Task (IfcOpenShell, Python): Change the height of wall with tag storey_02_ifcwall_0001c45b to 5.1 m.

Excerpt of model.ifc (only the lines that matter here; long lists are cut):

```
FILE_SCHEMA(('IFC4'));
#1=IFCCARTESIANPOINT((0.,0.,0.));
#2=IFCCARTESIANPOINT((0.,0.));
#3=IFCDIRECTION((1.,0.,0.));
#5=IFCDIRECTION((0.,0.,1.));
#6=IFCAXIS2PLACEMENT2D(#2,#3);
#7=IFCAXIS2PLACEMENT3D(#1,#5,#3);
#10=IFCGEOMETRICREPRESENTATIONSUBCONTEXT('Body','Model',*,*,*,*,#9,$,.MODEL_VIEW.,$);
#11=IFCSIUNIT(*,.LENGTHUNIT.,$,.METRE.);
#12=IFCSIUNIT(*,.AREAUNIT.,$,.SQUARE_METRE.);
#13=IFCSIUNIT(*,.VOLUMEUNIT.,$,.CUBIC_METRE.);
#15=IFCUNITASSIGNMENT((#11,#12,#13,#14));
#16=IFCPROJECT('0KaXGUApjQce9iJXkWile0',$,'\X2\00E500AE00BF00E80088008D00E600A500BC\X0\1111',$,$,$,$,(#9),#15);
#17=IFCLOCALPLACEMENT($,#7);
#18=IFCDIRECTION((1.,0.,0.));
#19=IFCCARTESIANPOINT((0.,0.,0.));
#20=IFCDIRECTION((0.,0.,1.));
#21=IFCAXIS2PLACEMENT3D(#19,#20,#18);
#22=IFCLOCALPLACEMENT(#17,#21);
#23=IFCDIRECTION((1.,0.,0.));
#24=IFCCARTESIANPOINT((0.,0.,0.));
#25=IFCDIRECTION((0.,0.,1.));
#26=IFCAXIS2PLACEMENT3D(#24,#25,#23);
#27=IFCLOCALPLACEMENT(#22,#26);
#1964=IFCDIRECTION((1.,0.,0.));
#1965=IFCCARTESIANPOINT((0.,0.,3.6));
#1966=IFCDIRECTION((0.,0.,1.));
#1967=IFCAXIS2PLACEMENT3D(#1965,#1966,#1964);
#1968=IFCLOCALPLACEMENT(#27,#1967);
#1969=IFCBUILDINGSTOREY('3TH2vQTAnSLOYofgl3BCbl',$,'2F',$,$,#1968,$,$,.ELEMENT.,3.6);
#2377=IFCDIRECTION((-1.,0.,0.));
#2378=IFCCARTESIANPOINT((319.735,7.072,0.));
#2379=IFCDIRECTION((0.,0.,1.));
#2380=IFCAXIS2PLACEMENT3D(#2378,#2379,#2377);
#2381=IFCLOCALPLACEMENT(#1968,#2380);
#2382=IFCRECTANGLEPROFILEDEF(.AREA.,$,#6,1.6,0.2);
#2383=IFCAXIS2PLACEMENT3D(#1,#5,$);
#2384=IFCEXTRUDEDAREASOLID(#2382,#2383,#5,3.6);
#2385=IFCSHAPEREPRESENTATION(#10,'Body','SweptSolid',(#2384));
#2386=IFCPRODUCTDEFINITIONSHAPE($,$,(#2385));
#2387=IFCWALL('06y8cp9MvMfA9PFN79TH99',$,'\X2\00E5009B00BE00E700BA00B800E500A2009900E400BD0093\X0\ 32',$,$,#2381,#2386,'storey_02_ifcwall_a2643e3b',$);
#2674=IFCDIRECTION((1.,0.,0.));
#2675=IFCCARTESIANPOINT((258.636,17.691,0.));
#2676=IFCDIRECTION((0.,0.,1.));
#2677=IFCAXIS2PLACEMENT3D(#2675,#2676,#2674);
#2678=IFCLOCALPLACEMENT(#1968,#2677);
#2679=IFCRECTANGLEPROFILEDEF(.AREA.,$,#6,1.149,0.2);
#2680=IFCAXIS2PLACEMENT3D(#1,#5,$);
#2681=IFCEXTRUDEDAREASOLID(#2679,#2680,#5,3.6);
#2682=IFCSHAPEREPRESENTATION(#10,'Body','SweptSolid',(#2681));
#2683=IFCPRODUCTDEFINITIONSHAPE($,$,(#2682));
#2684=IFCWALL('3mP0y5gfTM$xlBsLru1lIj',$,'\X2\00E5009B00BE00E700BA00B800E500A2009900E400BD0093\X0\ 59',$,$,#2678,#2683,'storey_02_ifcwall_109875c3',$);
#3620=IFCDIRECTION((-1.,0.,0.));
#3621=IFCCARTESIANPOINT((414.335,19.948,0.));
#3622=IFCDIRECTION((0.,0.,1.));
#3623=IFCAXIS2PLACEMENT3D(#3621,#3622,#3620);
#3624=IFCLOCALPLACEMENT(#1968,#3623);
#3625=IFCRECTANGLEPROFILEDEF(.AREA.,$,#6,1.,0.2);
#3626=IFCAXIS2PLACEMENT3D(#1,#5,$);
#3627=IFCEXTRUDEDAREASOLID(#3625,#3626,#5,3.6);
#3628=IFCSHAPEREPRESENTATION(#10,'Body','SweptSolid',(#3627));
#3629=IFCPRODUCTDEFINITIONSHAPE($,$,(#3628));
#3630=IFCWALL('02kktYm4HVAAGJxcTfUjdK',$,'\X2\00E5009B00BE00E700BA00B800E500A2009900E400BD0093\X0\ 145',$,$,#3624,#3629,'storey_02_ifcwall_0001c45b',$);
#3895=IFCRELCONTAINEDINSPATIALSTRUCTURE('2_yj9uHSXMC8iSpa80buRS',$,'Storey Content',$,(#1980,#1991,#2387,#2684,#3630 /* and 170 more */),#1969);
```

```python
import ifcopenshell
import ifcopenshell.geom
import ifcopenshell.util.representation
import ifcopenshell.util.shape
import ifcopenshell.util.unit

model = ifcopenshell.open("model.ifc")
unit_scale = ifcopenshell.util.unit.calculate_unit_scale(model)
settings = ifcopenshell.geom.settings()


def volume(element):
    """Net volume in cubic metres, openings subtracted."""
    shape = ifcopenshell.geom.create_shape(settings, element)
    return ifcopenshell.util.shape.get_volume(shape.geometry)


wall = model.by_id(3630)
before = volume(wall)

body = ifcopenshell.util.representation.get_representation(wall, "Model", "Body")
solid = body.Items[0]
old_height = solid.Depth
solid.Depth = 5.1 / unit_scale
after = volume(wall)

print(f"height {old_height:g} -> {solid.Depth:g}, volume {before:.3f} -> {after:.3f} m3")

model.write("model_rev.ifc")
```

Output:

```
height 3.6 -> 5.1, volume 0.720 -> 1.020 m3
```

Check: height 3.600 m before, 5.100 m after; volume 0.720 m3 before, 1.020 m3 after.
